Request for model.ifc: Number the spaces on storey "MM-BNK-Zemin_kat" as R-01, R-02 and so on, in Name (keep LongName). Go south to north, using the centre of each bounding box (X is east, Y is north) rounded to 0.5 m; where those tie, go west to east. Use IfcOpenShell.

First a look at what the model holds.

```python
import ifcopenshell
import ifcopenshell.util.element
import ifcopenshell.util.placement

model = ifcopenshell.open("model.ifc")
print(model.schema)
storey = next(s for s in model.by_type("IfcBuildingStorey") if s.Name == "MM-BNK-Zemin_kat")
spaces = [e for e in ifcopenshell.util.element.get_decomposition(storey) if e.is_a("IfcSpace")]
for e in sorted(spaces, key=lambda e: e.id()):
    origin = ifcopenshell.util.placement.get_local_placement(e.ObjectPlacement)[:3, 3]
    print(e.id(), e.Name, e.LongName, origin.round(2) + 0.0, sep=" | ")
```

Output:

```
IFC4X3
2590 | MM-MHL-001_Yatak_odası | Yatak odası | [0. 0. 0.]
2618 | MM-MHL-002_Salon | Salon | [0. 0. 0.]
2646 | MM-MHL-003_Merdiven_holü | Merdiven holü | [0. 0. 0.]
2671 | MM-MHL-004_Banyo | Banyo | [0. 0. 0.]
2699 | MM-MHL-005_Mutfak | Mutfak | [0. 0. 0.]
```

```python
import ifcopenshell
import ifcopenshell.geom
import ifcopenshell.util.element
import ifcopenshell.util.shape

model = ifcopenshell.open("model.ifc")
settings = ifcopenshell.geom.settings()
settings.set("use-world-coords", True)


def centre(element):
    shape = ifcopenshell.geom.create_shape(settings, element)
    return ifcopenshell.util.shape.get_bbox_centroid(shape.geometry)


storey = next(s for s in model.by_type("IfcBuildingStorey") if s.Name == "MM-BNK-Zemin_kat")
spaces = [e for e in ifcopenshell.util.element.get_decomposition(storey) if e.is_a("IfcSpace")]

# Insertion points can sit at a corner or the storey origin, so sort by the geometry (in metres).
centres = {e: centre(e) for e in spaces}
spaces.sort(key=lambda e: (round(centres[e][1] / 0.5), centres[e][0]))

for i, e in enumerate(spaces, start=1):
    number = f"R-{i:02d}"
    e.Name = number
    print(e.id(), number)

model.write("model_edited.ifc")
```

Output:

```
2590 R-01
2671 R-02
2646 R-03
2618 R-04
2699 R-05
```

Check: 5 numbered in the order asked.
